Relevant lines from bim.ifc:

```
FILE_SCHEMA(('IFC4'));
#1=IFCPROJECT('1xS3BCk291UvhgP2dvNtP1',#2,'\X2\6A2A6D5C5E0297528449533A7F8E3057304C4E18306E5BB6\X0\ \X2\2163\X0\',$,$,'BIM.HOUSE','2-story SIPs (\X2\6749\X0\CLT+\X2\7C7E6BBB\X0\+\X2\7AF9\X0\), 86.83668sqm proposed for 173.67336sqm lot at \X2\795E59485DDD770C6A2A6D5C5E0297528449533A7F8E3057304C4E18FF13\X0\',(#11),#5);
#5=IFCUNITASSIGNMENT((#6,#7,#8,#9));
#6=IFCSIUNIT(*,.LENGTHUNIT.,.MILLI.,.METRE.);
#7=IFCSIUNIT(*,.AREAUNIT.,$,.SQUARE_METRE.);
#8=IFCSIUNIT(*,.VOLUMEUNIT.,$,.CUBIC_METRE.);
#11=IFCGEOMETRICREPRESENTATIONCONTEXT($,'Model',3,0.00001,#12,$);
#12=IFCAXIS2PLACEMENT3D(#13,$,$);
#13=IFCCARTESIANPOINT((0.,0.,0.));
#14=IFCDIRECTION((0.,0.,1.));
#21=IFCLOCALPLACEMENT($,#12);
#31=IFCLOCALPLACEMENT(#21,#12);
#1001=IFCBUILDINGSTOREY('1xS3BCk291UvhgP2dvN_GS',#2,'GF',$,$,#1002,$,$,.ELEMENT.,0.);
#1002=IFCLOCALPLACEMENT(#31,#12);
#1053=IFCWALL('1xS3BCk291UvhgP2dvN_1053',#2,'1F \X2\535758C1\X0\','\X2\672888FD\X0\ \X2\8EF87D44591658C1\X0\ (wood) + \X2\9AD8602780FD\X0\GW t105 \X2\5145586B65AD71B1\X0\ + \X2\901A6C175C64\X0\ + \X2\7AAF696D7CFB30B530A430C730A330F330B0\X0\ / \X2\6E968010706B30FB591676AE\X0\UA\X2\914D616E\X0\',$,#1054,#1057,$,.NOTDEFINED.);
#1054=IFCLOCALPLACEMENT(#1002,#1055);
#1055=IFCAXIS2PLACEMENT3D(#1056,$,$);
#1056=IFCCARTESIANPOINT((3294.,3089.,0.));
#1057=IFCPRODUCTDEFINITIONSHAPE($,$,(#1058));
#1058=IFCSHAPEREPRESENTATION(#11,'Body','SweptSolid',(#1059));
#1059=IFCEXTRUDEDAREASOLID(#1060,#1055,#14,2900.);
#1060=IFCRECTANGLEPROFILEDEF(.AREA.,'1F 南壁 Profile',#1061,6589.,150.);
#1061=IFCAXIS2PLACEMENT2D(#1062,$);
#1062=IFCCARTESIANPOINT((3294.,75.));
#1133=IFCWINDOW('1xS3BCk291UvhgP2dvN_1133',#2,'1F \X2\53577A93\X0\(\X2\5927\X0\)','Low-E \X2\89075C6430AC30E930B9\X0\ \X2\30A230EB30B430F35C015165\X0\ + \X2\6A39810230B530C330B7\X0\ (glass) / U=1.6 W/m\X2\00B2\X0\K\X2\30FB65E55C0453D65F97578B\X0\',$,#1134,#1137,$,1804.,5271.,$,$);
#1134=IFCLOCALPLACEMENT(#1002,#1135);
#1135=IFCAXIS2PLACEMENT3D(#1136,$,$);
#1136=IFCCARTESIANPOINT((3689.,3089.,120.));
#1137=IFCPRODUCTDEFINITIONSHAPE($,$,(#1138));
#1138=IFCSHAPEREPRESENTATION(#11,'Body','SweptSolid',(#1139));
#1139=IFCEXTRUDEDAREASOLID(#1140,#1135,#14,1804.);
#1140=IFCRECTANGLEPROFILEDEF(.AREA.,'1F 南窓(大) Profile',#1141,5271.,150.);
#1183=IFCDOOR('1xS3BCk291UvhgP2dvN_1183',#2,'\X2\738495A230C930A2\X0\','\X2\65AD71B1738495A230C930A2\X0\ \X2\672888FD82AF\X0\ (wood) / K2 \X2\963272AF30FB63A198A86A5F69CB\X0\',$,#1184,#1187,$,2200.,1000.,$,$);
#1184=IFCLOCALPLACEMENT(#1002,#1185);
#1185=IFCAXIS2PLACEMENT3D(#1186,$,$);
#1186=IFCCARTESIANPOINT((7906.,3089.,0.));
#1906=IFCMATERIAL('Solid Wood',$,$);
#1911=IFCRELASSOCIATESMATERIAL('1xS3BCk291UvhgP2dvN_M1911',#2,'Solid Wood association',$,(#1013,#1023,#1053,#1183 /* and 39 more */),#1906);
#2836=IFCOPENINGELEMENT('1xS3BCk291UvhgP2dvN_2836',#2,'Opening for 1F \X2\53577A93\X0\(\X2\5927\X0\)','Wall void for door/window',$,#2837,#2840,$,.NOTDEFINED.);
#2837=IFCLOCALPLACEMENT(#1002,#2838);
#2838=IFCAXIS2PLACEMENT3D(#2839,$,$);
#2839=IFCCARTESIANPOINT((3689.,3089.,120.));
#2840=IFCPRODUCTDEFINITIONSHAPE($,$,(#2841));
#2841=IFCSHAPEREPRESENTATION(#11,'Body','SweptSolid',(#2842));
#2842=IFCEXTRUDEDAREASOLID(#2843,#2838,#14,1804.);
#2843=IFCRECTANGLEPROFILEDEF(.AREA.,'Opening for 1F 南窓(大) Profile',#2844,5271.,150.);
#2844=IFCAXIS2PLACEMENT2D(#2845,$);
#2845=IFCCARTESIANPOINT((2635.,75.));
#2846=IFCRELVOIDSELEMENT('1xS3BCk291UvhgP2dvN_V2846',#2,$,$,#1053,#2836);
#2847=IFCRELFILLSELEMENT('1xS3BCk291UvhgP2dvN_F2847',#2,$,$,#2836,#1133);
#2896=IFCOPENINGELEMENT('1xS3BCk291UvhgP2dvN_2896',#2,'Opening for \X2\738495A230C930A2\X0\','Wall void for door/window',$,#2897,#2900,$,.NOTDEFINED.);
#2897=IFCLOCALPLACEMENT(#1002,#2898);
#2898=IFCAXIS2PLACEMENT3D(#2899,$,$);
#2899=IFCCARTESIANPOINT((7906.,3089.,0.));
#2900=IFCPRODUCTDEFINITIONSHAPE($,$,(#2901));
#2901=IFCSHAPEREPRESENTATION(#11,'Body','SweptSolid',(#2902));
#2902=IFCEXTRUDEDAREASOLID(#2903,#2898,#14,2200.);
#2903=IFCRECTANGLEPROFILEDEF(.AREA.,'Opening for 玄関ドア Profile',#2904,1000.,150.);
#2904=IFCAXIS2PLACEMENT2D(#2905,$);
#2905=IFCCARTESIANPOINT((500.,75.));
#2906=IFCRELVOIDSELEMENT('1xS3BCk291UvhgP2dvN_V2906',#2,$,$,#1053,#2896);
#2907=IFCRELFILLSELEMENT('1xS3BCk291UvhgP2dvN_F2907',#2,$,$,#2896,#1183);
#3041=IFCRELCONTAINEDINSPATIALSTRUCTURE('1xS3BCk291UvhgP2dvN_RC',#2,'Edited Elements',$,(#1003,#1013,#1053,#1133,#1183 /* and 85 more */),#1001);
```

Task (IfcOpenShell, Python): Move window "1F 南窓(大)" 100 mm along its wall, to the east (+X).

```python
import ifcopenshell
import ifcopenshell.api.geometry
import ifcopenshell.util.placement

model = ifcopenshell.open("bim.ifc")

window = model.by_guid("1xS3BCk291UvhgP2dvN_1133")
opening = window.FillsVoids[0].RelatingOpeningElement
wall = opening.VoidsElements[0].RelatingBuildingElement

wall_matrix = ifcopenshell.util.placement.get_local_placement(wall.ObjectPlacement)
shift = wall_matrix[:3, 0] * 100.0
before = ifcopenshell.util.placement.get_local_placement(window.ObjectPlacement)[:3, 3].copy()

# The window is not placed relative to its opening, so move both.
for product in (opening, window):
    matrix = ifcopenshell.util.placement.get_local_placement(product.ObjectPlacement)
    matrix[:3, 3] += shift
    ifcopenshell.api.geometry.edit_object_placement(model, product=product, matrix=matrix, is_si=False)

after = ifcopenshell.util.placement.get_local_placement(window.ObjectPlacement)[:3, 3]
print("window moved by", (after - before).round(3) + 0.0)

model.write("bim_updated.ifc")
```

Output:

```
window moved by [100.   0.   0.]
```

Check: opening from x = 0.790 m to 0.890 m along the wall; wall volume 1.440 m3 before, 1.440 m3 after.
